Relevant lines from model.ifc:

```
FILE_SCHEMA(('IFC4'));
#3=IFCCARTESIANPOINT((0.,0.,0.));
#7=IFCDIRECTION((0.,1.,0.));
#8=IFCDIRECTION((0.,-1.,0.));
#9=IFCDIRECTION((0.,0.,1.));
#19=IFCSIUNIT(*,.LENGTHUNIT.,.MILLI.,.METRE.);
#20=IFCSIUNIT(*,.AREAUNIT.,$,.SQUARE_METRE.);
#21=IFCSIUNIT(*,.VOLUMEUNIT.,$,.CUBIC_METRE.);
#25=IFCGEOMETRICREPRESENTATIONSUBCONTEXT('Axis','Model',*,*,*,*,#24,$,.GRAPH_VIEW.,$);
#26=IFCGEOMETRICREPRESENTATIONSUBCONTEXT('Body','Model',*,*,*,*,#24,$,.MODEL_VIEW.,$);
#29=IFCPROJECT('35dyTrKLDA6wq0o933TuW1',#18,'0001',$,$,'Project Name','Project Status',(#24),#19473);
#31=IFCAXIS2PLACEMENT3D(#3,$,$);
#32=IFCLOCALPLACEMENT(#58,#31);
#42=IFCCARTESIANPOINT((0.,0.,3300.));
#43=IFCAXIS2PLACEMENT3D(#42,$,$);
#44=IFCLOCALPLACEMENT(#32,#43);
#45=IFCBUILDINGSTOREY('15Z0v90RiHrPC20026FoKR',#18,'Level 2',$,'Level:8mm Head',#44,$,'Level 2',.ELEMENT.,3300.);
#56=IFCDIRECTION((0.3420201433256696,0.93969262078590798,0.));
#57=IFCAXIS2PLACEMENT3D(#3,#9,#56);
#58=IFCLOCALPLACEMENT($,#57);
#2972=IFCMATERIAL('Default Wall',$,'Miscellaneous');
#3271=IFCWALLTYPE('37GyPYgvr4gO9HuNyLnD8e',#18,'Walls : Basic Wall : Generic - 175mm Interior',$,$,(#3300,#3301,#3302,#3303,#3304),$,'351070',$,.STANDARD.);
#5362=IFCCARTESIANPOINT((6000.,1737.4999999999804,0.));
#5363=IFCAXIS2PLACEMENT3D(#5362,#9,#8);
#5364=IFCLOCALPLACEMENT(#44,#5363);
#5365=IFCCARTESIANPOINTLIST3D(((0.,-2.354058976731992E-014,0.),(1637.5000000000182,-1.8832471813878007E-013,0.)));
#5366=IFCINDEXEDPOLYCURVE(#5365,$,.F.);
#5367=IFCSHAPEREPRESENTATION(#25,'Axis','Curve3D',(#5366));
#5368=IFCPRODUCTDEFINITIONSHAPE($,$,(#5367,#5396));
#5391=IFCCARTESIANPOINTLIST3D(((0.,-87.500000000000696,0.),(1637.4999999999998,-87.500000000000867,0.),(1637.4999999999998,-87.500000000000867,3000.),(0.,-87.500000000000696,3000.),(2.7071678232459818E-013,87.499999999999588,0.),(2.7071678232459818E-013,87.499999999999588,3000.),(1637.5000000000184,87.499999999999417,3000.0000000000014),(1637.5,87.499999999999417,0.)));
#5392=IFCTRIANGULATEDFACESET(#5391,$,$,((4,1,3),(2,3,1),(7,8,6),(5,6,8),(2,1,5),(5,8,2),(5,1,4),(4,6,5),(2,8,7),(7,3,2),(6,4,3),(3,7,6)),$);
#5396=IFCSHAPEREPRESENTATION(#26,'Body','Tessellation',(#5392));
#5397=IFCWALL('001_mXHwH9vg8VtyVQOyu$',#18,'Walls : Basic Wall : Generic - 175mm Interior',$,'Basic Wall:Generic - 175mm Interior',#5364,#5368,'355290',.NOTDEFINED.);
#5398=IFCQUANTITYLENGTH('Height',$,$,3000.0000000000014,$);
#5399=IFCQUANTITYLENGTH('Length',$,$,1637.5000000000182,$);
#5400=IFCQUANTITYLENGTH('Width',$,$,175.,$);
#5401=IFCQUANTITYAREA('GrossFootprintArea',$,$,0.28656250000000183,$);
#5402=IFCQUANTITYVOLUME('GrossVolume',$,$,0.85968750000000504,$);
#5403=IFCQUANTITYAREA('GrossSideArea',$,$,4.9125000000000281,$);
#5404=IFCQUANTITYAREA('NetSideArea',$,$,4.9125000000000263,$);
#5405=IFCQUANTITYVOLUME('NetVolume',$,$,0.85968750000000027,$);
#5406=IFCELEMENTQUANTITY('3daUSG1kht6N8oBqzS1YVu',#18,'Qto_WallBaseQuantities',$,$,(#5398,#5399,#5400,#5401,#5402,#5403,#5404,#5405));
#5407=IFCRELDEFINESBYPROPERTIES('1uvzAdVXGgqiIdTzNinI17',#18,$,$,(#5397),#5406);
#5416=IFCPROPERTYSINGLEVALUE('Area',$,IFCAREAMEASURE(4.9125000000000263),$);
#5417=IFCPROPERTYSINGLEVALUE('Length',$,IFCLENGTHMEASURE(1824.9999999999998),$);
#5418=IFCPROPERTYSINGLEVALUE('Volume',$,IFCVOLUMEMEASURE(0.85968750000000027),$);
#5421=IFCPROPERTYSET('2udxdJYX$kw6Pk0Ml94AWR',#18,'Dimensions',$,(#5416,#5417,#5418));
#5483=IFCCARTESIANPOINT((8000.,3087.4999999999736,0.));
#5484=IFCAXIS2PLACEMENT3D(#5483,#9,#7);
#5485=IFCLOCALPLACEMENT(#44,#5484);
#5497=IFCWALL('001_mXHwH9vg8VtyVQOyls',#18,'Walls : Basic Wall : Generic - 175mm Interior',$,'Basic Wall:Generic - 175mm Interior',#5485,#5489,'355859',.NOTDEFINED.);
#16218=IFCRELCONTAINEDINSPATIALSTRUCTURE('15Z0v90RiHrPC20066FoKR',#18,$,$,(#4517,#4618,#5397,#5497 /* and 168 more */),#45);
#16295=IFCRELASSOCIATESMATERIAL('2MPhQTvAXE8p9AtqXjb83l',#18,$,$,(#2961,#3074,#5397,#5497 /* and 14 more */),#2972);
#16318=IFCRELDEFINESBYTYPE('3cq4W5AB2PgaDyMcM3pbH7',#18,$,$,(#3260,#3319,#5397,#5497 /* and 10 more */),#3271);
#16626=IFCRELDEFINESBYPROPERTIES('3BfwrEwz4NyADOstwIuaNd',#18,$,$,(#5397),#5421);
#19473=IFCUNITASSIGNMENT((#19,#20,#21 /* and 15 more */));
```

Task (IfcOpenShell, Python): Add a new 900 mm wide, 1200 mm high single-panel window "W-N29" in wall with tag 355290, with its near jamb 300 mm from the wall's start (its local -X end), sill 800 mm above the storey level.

```python
import numpy as np
import ifcopenshell
import ifcopenshell.api.feature
import ifcopenshell.api.geometry
import ifcopenshell.api.pset
import ifcopenshell.api.root
import ifcopenshell.api.spatial
import ifcopenshell.geom
import ifcopenshell.util.element
import ifcopenshell.util.placement
import ifcopenshell.util.representation
import ifcopenshell.util.shape
import ifcopenshell.util.unit

model = ifcopenshell.open("model.ifc")
unit_scale = ifcopenshell.util.unit.calculate_unit_scale(model)
area_scale = ifcopenshell.util.unit.calculate_unit_scale(model, "AREAUNIT")
volume_scale = ifcopenshell.util.unit.calculate_unit_scale(model, "VOLUMEUNIT")
settings = ifcopenshell.geom.settings()


def volume(element):
    """Net volume in cubic metres, openings subtracted."""
    shape = ifcopenshell.geom.create_shape(settings, element)
    return ifcopenshell.util.shape.get_volume(shape.geometry)


wall = model.by_guid("001_mXHwH9vg8VtyVQOyu$")
storey = ifcopenshell.util.element.get_container(wall, ifc_class="IfcBuildingStorey")
context = ifcopenshell.util.representation.get_context(model, "Model", "Body", "MODEL_VIEW")
before = volume(wall)

width, height, from_end, sill = 0.9, 1.2, 0.3, 0.8  # metres

# The wall runs along its own X axis, and the end named is its -X end.
wall_shape = ifcopenshell.geom.create_shape(settings, wall)
x, y, z = ifcopenshell.util.shape.get_vertices(wall_shape.geometry).T
start = x.min() + from_end
face, thickness = float(y.min()), float(y.max() - y.min())
wall_matrix = ifcopenshell.util.placement.get_local_placement(wall.ObjectPlacement)
level = ifcopenshell.util.placement.get_local_placement(storey.ObjectPlacement)[2, 3]


def in_wall(x, y):
    """Placement at x, y metres in the wall's axes, at sill height."""
    matrix = wall_matrix.copy()
    matrix[:, 3] = wall_matrix @ np.array([x / unit_scale, y / unit_scale, 0.0, 1.0])
    matrix[2, 3] = level + sill / unit_scale
    return matrix


# Opening: a box that overshoots both wall faces by 50 mm.
opening = ifcopenshell.api.root.create_entity(model, ifc_class="IfcOpeningElement", predefined_type="OPENING")
box = ifcopenshell.api.geometry.add_wall_representation(
    model, context=context, length=width, height=height, thickness=thickness + 0.1
)
ifcopenshell.api.geometry.assign_representation(model, product=opening, representation=box)
ifcopenshell.api.geometry.edit_object_placement(model, product=opening, matrix=in_wall(start, face - 0.05), is_si=False)
ifcopenshell.api.feature.add_feature(model, feature=opening, element=wall)

window = ifcopenshell.api.root.create_entity(model, ifc_class="IfcWindow", name="W-N29", predefined_type="WINDOW")
window.OverallWidth, window.OverallHeight = width / unit_scale, height / unit_scale
window.PartitioningType = "SINGLE_PANEL"
body = ifcopenshell.api.geometry.add_window_representation(
    model,
    context=context,
    overall_width=window.OverallWidth,
    overall_height=window.OverallHeight,
    partition_type="SINGLE_PANEL",
)
ifcopenshell.api.geometry.assign_representation(model, product=window, representation=body)
ifcopenshell.api.spatial.assign_container(model, products=[window], relating_structure=storey)
ifcopenshell.api.feature.add_filling(model, opening=opening, element=window)

# Centre the window in the wall's thickness.
ifcopenshell.api.geometry.edit_object_placement(model, product=window, matrix=in_wall(start, face), is_si=False)
window_shape = ifcopenshell.geom.create_shape(settings, window)
depth = ifcopenshell.util.shape.get_vertices(window_shape.geometry)[:, 1]
offset = face + thickness / 2 - (depth.min() + depth.max()) / 2
ifcopenshell.api.geometry.edit_object_placement(model, product=window, matrix=in_wall(start, offset), is_si=False)

after = volume(wall)

# Update the wall's stored quantities.
qto = model.by_id(ifcopenshell.util.element.get_pset(wall, "Qto_WallBaseQuantities", should_inherit=False)["id"])
ifcopenshell.api.pset.edit_qto(model, qto=qto, properties={
    "NetSideArea": after / thickness / area_scale,
    "NetVolume": after / volume_scale,
})
pset = model.by_id(ifcopenshell.util.element.get_pset(wall, "Dimensions", should_inherit=False)["id"])
ifcopenshell.api.pset.edit_pset(model, pset=pset, properties={
    "Area": model.create_entity("IfcAreaMeasure", after / thickness / area_scale),
    "Volume": model.create_entity("IfcVolumeMeasure", after / volume_scale),
})

print(f"wall volume {before:.3f} -> {after:.3f} m3")

model.write("model_rev.ifc")
```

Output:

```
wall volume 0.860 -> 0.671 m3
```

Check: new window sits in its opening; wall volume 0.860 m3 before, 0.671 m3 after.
